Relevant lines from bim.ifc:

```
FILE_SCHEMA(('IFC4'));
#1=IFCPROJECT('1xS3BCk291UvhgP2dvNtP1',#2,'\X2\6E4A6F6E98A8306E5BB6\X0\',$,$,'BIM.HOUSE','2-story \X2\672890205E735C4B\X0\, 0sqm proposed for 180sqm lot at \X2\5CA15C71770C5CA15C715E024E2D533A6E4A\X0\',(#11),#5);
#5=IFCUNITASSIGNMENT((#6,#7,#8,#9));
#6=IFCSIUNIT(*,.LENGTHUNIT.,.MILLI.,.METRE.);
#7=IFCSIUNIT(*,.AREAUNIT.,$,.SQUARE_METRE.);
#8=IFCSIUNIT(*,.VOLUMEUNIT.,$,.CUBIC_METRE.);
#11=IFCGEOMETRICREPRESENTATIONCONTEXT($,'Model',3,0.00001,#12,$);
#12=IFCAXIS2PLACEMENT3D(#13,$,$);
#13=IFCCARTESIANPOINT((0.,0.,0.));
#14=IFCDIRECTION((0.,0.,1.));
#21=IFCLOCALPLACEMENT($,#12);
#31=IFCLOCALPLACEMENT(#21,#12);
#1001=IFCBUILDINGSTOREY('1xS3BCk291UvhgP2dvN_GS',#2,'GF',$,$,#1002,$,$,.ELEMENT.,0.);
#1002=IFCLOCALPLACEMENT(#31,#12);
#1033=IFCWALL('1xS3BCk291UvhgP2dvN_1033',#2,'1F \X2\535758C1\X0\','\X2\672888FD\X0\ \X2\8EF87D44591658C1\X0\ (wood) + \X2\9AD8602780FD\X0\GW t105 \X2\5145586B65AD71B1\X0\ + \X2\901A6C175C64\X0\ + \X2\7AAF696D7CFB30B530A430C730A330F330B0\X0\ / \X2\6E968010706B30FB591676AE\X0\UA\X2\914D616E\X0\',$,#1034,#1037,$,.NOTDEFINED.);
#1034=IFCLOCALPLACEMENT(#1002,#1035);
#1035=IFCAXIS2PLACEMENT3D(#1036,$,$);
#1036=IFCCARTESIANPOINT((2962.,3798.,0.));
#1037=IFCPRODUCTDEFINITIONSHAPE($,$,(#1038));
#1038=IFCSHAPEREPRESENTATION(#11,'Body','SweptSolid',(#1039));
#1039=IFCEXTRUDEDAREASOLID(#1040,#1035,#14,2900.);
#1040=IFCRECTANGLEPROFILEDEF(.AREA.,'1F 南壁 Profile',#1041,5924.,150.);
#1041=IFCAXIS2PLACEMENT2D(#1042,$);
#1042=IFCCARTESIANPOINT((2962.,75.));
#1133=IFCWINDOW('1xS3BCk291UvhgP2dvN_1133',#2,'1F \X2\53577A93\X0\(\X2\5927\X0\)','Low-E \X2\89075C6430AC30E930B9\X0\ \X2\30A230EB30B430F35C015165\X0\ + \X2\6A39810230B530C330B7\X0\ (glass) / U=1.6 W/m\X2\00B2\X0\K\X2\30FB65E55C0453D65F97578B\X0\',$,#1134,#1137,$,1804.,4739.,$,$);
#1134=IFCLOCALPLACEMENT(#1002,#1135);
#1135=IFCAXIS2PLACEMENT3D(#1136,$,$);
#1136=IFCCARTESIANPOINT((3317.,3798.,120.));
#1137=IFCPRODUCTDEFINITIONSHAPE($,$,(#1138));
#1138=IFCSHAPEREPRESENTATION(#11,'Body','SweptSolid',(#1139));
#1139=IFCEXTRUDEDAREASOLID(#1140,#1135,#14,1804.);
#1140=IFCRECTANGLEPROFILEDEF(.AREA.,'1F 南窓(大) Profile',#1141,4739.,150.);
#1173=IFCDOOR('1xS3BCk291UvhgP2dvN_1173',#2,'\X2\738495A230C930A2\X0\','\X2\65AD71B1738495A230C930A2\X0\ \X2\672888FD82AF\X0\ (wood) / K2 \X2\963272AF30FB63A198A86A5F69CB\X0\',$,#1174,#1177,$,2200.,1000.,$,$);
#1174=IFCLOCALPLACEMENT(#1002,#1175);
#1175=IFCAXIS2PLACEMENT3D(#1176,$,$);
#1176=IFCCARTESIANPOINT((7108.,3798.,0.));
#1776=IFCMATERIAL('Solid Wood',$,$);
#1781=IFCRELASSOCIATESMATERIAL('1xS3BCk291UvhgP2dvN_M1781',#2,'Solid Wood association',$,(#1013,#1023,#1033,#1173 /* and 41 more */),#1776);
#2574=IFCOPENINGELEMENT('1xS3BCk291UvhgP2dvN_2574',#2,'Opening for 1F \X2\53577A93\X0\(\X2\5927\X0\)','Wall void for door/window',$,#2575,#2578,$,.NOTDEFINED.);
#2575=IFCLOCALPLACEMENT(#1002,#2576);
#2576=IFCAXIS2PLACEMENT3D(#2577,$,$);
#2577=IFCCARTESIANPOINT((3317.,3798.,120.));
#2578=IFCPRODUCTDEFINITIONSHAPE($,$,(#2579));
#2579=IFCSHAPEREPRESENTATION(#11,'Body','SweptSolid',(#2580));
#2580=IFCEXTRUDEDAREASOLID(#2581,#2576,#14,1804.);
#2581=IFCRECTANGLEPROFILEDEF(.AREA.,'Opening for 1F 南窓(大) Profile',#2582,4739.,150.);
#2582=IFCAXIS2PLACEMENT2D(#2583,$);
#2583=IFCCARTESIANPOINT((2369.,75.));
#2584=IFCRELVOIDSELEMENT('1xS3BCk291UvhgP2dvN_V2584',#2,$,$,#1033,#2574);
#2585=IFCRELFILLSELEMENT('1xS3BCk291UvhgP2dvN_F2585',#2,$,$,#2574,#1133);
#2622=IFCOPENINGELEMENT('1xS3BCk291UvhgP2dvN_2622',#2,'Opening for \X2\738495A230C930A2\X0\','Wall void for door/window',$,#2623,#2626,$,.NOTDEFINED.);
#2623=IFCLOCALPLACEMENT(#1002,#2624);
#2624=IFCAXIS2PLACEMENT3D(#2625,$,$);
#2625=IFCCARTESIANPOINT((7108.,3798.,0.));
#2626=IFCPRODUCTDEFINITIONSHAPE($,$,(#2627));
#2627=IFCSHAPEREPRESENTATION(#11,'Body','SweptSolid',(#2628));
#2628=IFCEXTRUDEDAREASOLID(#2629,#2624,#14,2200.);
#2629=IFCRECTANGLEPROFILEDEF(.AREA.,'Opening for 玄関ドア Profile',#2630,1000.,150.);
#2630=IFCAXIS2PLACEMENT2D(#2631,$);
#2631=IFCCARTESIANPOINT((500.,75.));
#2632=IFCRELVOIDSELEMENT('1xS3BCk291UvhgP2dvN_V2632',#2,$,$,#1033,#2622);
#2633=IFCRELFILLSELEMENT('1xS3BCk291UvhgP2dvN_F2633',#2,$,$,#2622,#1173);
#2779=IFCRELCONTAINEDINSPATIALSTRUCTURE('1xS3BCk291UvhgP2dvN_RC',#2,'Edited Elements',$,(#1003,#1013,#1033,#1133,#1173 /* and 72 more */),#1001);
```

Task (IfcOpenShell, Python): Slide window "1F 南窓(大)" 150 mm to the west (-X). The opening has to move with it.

```python
import ifcopenshell
import ifcopenshell.api.geometry
import ifcopenshell.util.placement

model = ifcopenshell.open("bim.ifc")

window = model.by_id(1133)
opening = window.FillsVoids[0].RelatingOpeningElement
wall = opening.VoidsElements[0].RelatingBuildingElement

wall_matrix = ifcopenshell.util.placement.get_local_placement(wall.ObjectPlacement)
shift = wall_matrix[:3, 0] * -150.0
before = ifcopenshell.util.placement.get_local_placement(window.ObjectPlacement)[:3, 3].copy()

# The window is not placed relative to its opening, so move both.
for product in (opening, window):
    matrix = ifcopenshell.util.placement.get_local_placement(product.ObjectPlacement)
    matrix[:3, 3] += shift
    ifcopenshell.api.geometry.edit_object_placement(model, product=product, matrix=matrix, is_si=False)

after = ifcopenshell.util.placement.get_local_placement(window.ObjectPlacement)[:3, 3]
print("window moved by", (after - before).round(3) + 0.0)

model.write("bim_v2.ifc")
```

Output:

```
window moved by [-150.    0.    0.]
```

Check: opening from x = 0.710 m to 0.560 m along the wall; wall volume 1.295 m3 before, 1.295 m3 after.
